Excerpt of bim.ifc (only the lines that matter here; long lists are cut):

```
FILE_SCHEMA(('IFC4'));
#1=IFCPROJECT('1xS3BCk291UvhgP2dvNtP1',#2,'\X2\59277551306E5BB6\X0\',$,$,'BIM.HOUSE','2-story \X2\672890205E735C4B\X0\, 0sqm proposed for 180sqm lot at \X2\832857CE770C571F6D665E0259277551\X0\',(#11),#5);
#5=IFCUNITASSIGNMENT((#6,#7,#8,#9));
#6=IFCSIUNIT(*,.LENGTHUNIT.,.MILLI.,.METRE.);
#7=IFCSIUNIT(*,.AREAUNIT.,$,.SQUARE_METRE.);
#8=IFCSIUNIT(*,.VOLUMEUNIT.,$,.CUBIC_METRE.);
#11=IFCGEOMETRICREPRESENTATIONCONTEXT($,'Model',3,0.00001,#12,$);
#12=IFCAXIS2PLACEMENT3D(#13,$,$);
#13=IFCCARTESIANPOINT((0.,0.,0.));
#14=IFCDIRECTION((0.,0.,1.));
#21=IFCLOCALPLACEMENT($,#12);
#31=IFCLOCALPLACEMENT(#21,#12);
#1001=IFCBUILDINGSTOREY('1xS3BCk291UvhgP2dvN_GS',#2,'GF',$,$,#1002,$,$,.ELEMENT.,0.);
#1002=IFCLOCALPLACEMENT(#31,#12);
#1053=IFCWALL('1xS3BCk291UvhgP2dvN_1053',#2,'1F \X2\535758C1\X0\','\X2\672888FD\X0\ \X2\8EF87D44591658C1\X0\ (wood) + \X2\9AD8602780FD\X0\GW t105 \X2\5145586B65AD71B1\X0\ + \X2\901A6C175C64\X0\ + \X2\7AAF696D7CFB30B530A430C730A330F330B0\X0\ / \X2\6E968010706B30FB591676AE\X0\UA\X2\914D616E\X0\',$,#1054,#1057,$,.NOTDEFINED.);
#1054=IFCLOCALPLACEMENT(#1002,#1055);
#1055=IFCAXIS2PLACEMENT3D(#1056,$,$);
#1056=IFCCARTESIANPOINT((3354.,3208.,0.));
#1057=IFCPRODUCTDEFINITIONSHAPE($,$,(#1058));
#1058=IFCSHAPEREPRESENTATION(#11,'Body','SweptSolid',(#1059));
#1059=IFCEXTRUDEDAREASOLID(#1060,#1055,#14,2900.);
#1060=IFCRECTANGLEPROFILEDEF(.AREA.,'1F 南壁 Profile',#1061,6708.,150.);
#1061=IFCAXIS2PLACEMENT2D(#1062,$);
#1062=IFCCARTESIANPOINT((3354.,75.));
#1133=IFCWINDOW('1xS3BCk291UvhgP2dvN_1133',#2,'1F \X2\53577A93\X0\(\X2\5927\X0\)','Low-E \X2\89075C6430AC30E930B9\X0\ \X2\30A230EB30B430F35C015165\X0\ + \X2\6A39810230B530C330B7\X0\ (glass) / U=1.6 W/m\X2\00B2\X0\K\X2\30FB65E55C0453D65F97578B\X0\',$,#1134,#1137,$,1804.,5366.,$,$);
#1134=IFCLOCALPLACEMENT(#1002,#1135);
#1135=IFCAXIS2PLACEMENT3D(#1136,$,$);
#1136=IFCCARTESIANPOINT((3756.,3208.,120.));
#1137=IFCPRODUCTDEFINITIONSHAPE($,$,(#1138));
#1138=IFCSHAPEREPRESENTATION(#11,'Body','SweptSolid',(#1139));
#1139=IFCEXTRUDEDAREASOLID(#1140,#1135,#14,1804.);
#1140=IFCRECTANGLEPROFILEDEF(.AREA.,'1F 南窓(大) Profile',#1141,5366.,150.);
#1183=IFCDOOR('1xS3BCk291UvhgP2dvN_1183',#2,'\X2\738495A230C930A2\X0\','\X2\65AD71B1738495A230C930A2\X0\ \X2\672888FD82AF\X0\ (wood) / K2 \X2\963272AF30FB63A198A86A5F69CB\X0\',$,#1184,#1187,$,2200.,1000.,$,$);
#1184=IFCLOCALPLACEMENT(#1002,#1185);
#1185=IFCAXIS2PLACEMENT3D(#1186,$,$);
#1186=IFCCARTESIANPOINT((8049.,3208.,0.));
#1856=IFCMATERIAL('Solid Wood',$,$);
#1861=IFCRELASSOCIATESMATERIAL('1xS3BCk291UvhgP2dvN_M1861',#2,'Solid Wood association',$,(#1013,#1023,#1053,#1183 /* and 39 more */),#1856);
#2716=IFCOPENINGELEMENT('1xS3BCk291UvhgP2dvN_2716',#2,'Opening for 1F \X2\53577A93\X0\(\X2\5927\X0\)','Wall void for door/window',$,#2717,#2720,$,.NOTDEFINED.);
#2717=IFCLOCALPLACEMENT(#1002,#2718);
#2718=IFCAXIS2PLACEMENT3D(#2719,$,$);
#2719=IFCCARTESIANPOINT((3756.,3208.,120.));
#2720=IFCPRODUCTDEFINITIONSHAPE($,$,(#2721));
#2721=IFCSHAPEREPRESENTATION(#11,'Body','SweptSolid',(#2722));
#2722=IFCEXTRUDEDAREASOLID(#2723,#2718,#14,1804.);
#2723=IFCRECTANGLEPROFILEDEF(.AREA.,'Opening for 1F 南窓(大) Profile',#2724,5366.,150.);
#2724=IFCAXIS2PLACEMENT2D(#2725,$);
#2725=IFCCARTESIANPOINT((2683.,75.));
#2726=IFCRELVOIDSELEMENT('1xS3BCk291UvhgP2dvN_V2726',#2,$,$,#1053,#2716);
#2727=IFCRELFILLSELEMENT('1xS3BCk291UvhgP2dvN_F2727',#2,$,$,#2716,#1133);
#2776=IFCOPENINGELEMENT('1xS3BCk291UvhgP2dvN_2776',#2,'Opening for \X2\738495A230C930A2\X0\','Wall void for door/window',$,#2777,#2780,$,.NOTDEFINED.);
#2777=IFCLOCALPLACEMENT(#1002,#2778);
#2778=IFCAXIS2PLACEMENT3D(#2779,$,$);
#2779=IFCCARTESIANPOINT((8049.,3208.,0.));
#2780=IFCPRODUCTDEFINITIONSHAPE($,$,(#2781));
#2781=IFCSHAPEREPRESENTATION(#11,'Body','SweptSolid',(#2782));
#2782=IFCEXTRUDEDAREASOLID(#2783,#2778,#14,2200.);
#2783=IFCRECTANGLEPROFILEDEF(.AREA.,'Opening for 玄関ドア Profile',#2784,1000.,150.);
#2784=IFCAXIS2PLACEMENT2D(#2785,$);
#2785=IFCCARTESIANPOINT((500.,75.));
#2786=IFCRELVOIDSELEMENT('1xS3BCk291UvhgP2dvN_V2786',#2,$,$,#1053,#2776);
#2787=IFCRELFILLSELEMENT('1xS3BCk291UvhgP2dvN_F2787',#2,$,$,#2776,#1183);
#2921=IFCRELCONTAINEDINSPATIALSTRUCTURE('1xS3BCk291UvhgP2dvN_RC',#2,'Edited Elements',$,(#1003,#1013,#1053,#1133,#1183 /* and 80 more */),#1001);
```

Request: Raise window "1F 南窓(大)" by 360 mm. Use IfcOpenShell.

```python
import numpy as np
import ifcopenshell
import ifcopenshell.api.geometry
import ifcopenshell.util.placement
import ifcopenshell.util.unit

model = ifcopenshell.open("bim.ifc")
unit_scale = ifcopenshell.util.unit.calculate_unit_scale(model)

window = model.by_guid("1xS3BCk291UvhgP2dvN_1133")
opening = window.FillsVoids[0].RelatingOpeningElement
dz = 0.36 / unit_scale

shift = np.array([0.0, 0.0, dz])
# The window is not placed relative to its opening, so move both.
for product in (opening, window):
    matrix = ifcopenshell.util.placement.get_local_placement(product.ObjectPlacement)
    matrix[:3, 3] += shift
    ifcopenshell.api.geometry.edit_object_placement(model, product=product, matrix=matrix, is_si=False)

print(f"moved by {dz * unit_scale:+.3f} m")

model.write("bim_updated.ifc")
```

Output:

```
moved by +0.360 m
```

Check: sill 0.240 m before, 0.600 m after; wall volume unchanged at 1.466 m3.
